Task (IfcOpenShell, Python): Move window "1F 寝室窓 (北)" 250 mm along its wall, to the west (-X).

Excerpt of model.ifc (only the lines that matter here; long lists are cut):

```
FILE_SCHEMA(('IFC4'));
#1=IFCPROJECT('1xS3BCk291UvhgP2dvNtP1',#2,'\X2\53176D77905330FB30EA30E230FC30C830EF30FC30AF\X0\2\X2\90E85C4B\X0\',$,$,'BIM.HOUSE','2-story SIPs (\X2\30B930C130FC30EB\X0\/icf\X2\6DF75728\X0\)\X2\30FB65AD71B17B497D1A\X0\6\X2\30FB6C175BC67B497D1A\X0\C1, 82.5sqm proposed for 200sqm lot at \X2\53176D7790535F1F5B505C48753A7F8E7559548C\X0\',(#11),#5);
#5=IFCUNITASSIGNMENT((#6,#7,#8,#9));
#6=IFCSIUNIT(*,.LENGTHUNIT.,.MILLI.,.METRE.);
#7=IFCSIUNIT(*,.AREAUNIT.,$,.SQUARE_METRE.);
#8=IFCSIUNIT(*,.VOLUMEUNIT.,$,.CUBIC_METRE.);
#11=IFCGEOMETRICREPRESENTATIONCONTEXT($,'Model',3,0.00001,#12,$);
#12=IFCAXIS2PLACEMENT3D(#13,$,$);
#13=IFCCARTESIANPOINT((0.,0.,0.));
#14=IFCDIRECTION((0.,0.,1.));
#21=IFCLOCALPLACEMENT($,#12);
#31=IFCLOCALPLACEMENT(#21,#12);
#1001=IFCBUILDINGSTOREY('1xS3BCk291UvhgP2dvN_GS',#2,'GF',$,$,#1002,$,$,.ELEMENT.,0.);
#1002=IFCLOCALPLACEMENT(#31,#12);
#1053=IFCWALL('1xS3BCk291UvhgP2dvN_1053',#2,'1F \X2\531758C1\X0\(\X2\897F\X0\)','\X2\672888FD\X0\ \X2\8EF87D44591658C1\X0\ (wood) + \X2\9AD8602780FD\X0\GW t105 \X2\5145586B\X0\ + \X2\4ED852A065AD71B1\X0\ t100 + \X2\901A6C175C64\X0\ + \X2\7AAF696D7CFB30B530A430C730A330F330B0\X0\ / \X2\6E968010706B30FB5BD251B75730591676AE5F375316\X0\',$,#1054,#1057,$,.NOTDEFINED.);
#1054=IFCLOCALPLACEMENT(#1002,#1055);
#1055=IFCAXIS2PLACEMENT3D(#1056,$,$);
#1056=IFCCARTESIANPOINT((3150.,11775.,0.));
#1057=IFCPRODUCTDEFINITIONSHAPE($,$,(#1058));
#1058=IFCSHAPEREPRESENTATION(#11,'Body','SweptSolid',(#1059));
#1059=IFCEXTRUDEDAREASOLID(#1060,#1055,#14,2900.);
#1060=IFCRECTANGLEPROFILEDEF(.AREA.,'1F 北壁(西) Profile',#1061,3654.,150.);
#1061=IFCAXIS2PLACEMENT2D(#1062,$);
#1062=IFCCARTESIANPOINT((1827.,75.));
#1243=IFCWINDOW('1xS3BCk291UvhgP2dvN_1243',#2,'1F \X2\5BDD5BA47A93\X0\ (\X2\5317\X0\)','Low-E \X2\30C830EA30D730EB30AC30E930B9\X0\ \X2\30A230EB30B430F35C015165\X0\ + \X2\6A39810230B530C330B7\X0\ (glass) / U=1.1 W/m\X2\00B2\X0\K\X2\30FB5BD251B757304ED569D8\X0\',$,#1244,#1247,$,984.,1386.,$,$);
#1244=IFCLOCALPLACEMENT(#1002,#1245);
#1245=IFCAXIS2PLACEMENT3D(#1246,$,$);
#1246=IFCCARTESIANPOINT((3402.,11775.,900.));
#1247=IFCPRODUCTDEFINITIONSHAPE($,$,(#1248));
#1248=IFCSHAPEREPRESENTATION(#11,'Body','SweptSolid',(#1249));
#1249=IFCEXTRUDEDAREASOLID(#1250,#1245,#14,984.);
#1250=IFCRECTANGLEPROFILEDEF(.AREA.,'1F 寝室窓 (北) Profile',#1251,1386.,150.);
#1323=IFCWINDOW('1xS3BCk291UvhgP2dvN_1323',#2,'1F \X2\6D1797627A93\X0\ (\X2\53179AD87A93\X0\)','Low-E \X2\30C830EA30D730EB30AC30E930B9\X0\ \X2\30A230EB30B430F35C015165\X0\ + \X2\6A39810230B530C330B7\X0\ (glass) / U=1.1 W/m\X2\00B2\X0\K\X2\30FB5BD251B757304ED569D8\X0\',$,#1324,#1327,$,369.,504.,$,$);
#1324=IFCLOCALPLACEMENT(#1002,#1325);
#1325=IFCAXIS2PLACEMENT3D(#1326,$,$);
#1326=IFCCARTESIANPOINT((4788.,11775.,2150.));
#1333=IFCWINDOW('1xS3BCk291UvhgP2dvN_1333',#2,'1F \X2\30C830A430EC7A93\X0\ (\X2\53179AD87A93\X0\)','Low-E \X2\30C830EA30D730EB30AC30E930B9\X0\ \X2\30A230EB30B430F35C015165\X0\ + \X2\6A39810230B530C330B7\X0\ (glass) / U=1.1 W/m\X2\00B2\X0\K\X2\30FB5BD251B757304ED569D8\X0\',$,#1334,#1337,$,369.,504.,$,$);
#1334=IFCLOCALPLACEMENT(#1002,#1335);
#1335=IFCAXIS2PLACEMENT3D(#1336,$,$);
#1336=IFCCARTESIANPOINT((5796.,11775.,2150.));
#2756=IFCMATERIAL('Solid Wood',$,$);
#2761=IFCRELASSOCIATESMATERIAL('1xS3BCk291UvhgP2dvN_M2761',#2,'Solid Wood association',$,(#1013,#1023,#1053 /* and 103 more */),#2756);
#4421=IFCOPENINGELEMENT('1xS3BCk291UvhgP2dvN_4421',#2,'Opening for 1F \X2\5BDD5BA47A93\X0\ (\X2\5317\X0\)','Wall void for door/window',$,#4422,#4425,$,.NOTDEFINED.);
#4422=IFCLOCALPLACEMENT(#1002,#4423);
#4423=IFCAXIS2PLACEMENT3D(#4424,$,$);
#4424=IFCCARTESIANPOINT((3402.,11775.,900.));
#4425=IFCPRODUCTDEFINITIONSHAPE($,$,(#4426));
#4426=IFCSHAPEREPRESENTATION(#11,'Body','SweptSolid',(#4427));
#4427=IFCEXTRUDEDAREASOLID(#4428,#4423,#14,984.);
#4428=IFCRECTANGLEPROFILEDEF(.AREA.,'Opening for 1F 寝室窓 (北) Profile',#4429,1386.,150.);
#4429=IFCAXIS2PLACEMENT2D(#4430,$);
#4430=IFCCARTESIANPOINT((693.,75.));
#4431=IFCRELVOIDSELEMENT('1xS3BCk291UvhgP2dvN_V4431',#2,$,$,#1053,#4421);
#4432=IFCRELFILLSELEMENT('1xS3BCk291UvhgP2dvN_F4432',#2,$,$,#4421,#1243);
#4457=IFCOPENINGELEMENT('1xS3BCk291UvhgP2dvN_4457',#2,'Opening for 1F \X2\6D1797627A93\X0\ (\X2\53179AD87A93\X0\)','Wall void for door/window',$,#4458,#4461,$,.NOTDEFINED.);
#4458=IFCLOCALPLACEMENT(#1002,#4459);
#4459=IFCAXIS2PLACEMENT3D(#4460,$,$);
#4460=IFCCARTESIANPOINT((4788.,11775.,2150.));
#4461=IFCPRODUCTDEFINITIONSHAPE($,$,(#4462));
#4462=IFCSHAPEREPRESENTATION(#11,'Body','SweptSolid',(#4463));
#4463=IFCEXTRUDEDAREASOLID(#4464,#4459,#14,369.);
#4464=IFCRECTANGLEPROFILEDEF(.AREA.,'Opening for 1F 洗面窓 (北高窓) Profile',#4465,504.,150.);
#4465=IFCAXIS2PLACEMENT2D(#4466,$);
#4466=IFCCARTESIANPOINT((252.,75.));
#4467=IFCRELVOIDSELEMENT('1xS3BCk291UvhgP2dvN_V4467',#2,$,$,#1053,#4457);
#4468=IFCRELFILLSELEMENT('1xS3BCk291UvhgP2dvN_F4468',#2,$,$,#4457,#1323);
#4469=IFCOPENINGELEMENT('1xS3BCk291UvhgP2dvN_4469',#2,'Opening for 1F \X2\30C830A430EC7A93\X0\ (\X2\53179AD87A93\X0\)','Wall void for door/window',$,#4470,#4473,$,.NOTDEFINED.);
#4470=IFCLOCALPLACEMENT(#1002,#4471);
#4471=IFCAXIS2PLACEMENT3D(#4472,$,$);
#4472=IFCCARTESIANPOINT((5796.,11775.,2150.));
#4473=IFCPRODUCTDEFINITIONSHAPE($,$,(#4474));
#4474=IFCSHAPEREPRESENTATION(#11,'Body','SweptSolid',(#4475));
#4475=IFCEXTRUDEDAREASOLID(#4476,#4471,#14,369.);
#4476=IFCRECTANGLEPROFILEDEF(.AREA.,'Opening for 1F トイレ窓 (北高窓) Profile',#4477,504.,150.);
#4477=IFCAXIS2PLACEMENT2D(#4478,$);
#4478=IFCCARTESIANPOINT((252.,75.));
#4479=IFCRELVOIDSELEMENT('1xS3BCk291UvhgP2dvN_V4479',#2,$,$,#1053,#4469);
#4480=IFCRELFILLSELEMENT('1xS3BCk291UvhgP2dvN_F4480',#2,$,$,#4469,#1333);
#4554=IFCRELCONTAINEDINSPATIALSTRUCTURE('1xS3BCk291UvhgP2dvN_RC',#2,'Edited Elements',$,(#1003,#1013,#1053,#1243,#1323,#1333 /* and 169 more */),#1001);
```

```python
import ifcopenshell
import ifcopenshell.api.geometry
import ifcopenshell.util.placement
import ifcopenshell.util.unit

model = ifcopenshell.open("model.ifc")
unit_scale = ifcopenshell.util.unit.calculate_unit_scale(model)

window = model.by_guid("1xS3BCk291UvhgP2dvN_1243")
opening = window.FillsVoids[0].RelatingOpeningElement
wall = opening.VoidsElements[0].RelatingBuildingElement

wall_matrix = ifcopenshell.util.placement.get_local_placement(wall.ObjectPlacement)
shift = wall_matrix[:3, 0] * -0.25 / unit_scale
before = ifcopenshell.util.placement.get_local_placement(window.ObjectPlacement)[:3, 3].copy()

# The window is not placed relative to its opening, so move both.
for product in (opening, window):
    matrix = ifcopenshell.util.placement.get_local_placement(product.ObjectPlacement)
    matrix[:3, 3] += shift
    ifcopenshell.api.geometry.edit_object_placement(model, product=product, matrix=matrix, is_si=False)

after = ifcopenshell.util.placement.get_local_placement(window.ObjectPlacement)[:3, 3]
print("window moved by", (after - before).round(3) + 0.0)

model.write("model_edited.ifc")
```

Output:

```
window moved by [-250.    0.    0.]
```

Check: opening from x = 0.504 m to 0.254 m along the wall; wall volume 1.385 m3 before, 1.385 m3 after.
